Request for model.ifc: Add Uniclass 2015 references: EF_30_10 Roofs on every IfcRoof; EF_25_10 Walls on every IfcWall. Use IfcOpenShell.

First a look at what the model holds.

```python
import ifcopenshell

model = ifcopenshell.open("model.ifc")
print(model.schema)
print("classifications:", [c.Name for c in model.by_type("IfcClassification")])
for ifc_class in ("IfcDoor", "IfcRoof", "IfcStair", "IfcWall", "IfcWindow"):
    print(ifc_class, len(model.by_type(ifc_class)))
```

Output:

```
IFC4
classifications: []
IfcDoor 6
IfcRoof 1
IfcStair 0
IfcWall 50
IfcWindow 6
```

```python
import ifcopenshell
import ifcopenshell.api.classification

model = ifcopenshell.open("model.ifc")

system = ifcopenshell.api.classification.add_classification(model, classification="Uniclass 2015")

codes = {
    "IfcRoof": ("EF_30_10", "Roofs"),
    "IfcWall": ("EF_25_10", "Walls"),
}
for ifc_class, (code, name) in codes.items():
    products = model.by_type(ifc_class)
    ifcopenshell.api.classification.add_reference(
        model, products=products, classification=system, identification=code, name=name
    )
    print(code, len(products))

model.write("model_v2.ifc")
```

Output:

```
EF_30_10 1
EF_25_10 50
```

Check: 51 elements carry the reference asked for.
